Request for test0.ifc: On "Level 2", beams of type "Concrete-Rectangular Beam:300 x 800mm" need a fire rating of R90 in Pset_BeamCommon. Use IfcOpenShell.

First a look at what the model holds.

```python
import ifcopenshell
import ifcopenshell.util.element

model = ifcopenshell.open("test0.ifc")
print(model.schema)
storey = next(s for s in model.by_type("IfcBuildingStorey") if s.Name == "Level 2")
beams = [e for e in ifcopenshell.util.element.get_decomposition(storey) if e.is_a("IfcBeam")]
seen = {}
for e in beams:
    element_type = ifcopenshell.util.element.get_type(e)
    key = (element_type.Name if element_type != e and element_type else None, ifcopenshell.util.element.get_pset(e, "Pset_BeamCommon", "FireRating"))
    seen[key] = seen.get(key, 0) + 1
for (name, value), count in sorted(seen.items(), key=str):
    print(count, "x", name, "|", value)
```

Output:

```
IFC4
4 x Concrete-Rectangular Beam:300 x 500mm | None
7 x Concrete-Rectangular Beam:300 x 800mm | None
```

```python
import ifcopenshell
import ifcopenshell.api.pset
import ifcopenshell.util.element

model = ifcopenshell.open("test0.ifc")

storey = next(s for s in model.by_type("IfcBuildingStorey") if s.Name == "Level 2")
beams = [e for e in ifcopenshell.util.element.get_decomposition(storey) if e.is_a("IfcBeam")]

count = 0
for e in beams:
    element_type = ifcopenshell.util.element.get_type(e)
    if element_type in (None, e) or element_type.Name != "Concrete-Rectangular Beam:300 x 800mm":
        continue
    # add_pset returns the element's existing set when there is one.
    pset = ifcopenshell.api.pset.add_pset(model, product=e, name="Pset_BeamCommon")
    ifcopenshell.api.pset.edit_pset(model, pset=pset, properties={"FireRating": "R90"})
    count += 1

print(count, "beams updated")

model.write("test0_v2.ifc")
```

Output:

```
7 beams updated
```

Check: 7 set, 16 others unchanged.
